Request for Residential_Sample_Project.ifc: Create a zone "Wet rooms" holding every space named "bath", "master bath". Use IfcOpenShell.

First a look at what the model holds.

```python
import ifcopenshell

model = ifcopenshell.open("Residential_Sample_Project.ifc")
print(model.schema)
seen = {}
for space in model.by_type("IfcSpace"):
    seen[space.LongName] = seen.get(space.LongName, 0) + 1
for name, count in sorted(seen.items(), key=str):
    print(count, "x", name)
print("zones:", [z.Name for z in model.by_type("IfcZone")][:20])
```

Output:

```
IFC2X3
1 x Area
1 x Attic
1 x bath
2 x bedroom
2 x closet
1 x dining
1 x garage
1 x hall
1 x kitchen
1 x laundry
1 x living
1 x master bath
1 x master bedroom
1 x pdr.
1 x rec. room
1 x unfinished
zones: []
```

```python
import ifcopenshell
import ifcopenshell.api.group
import ifcopenshell.api.root

model = ifcopenshell.open("Residential_Sample_Project.ifc")

names = {"bath", "master bath"}
spaces = [s for s in model.by_type("IfcSpace") if s.LongName in names]

zone = ifcopenshell.api.root.create_entity(model, ifc_class="IfcZone", name="Wet rooms")
ifcopenshell.api.group.assign_group(model, products=spaces, group=zone)
print(len(spaces), "spaces in", zone.Name)

model.write("Residential_Sample_Project_updated.ifc")
```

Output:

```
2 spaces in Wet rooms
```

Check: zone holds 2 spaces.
